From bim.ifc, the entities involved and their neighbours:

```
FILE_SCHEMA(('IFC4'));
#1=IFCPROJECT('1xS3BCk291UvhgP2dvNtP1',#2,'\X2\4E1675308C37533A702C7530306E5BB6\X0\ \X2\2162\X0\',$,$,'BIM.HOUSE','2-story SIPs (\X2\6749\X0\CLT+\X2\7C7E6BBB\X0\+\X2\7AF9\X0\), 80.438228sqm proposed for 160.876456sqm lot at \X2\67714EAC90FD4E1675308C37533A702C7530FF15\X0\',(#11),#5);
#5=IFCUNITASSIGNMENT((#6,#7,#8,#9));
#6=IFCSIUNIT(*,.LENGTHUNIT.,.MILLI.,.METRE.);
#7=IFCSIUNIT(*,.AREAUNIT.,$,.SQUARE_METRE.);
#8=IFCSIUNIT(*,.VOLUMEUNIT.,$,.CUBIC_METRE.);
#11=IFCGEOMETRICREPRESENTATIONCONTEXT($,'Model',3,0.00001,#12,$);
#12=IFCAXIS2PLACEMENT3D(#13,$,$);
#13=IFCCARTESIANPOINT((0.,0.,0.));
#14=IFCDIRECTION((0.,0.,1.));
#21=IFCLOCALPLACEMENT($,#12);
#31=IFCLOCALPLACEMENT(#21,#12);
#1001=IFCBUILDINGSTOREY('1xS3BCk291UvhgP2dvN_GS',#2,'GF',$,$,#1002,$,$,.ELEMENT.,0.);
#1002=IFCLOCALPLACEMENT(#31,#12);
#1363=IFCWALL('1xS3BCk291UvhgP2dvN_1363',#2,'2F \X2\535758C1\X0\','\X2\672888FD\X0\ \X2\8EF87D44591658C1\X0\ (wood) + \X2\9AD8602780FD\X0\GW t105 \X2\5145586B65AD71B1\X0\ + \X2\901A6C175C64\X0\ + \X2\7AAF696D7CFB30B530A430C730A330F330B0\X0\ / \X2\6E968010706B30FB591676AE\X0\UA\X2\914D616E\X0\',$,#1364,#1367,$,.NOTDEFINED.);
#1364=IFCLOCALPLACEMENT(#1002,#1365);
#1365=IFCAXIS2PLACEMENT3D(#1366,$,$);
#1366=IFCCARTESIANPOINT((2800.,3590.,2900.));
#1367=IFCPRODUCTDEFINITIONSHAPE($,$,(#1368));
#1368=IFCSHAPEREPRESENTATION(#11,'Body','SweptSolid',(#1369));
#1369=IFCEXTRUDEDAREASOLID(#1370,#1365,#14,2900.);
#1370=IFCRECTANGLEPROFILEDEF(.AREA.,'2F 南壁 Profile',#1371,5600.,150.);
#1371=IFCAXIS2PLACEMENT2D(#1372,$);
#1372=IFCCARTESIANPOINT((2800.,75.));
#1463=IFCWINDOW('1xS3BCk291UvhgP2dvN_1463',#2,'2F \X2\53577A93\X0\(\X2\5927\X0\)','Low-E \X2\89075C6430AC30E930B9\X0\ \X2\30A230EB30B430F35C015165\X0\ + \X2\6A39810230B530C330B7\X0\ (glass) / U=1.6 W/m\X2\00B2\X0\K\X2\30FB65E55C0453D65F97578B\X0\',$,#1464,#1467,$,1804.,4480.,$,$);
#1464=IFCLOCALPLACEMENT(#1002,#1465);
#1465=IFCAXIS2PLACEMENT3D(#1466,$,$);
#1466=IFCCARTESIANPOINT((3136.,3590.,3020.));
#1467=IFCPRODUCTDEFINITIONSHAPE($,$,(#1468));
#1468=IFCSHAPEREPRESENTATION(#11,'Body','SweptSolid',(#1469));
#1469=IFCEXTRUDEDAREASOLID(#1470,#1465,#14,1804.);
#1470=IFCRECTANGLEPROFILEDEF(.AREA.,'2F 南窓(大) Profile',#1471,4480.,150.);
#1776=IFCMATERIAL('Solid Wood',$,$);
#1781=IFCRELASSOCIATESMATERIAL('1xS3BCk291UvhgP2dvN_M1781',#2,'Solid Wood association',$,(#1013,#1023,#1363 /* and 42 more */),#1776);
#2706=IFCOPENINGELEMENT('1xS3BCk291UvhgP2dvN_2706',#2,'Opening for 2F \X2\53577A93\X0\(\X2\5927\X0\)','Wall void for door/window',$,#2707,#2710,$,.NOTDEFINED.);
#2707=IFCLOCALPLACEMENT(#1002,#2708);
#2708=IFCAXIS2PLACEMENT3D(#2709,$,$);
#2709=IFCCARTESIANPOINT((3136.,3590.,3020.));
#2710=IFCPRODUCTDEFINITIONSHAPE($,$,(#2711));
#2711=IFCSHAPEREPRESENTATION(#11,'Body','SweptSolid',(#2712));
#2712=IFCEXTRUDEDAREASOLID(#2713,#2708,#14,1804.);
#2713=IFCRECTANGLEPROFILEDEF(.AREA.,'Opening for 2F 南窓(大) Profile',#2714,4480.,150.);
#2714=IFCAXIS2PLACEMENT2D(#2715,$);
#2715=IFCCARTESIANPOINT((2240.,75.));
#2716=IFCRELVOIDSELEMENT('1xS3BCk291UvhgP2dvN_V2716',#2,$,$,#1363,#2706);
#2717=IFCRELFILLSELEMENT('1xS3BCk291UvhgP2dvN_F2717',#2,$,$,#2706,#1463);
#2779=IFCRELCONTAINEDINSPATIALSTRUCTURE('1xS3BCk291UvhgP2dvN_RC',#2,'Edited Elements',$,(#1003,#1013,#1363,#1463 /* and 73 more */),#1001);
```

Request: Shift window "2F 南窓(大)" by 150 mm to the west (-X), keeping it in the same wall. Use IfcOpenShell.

```python
import ifcopenshell
import ifcopenshell.api.geometry
import ifcopenshell.util.placement
import ifcopenshell.util.unit

model = ifcopenshell.open("bim.ifc")
unit_scale = ifcopenshell.util.unit.calculate_unit_scale(model)

window = model.by_guid("1xS3BCk291UvhgP2dvN_1463")
opening = window.FillsVoids[0].RelatingOpeningElement
wall = opening.VoidsElements[0].RelatingBuildingElement

wall_matrix = ifcopenshell.util.placement.get_local_placement(wall.ObjectPlacement)
shift = wall_matrix[:3, 0] * -0.15 / unit_scale
before = ifcopenshell.util.placement.get_local_placement(window.ObjectPlacement)[:3, 3].copy()

# The window is not placed relative to its opening, so move both.
for product in (opening, window):
    matrix = ifcopenshell.util.placement.get_local_placement(product.ObjectPlacement)
    matrix[:3, 3] += shift
    ifcopenshell.api.geometry.edit_object_placement(model, product=product, matrix=matrix, is_si=False)

after = ifcopenshell.util.placement.get_local_placement(window.ObjectPlacement)[:3, 3]
print("window moved by", (after - before).round(3) + 0.0)

model.write("bim_v2.ifc")
```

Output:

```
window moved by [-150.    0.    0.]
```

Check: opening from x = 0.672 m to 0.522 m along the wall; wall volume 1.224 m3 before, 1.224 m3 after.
